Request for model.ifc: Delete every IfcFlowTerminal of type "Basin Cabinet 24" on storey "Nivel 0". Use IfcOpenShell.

First a look at what the model holds.

```python
import ifcopenshell
import ifcopenshell.util.element

model = ifcopenshell.open("model.ifc")
print(model.schema)
storey = next(s for s in model.by_type("IfcBuildingStorey") if s.Name == "Nivel 0")
terminals = [e for e in ifcopenshell.util.element.get_decomposition(storey) if e.is_a("IfcFlowTerminal")]
seen = {}
for e in terminals:
    element_type = ifcopenshell.util.element.get_type(e)
    name = element_type.Name if element_type not in (None, e) else None
    seen[name] = seen.get(name, 0) + 1
for name, count in sorted(seen.items(), key=str):
    print(count, "x", name)
```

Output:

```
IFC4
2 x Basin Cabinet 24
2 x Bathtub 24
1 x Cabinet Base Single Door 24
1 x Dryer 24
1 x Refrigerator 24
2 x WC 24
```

```python
import ifcopenshell
import ifcopenshell.api.root
import ifcopenshell.util.element

model = ifcopenshell.open("model.ifc")

storey = next(s for s in model.by_type("IfcBuildingStorey") if s.Name == "Nivel 0")
terminals = [e for e in ifcopenshell.util.element.get_decomposition(storey) if e.is_a("IfcFlowTerminal")]
targets = [e for e in terminals if (t := ifcopenshell.util.element.get_type(e)) not in (None, e) and t.Name == "Basin Cabinet 24"]

for e in targets:
    ifcopenshell.api.root.remove_product(model, product=e)
print(len(targets), "removed")

model.write("model_edited.ifc")
```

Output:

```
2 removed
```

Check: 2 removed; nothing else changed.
